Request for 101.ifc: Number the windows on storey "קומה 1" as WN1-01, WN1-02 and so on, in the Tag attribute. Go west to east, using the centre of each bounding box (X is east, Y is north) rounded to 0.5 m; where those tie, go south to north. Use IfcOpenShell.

First a look at what the model holds.

```python
import ifcopenshell
import ifcopenshell.util.element
import ifcopenshell.util.placement

model = ifcopenshell.open("101.ifc")
print(model.schema)
storey = next(s for s in model.by_type("IfcBuildingStorey") if s.Name == "קומה 1")
windows = [e for e in ifcopenshell.util.element.get_decomposition(storey) if e.is_a("IfcWindow")]
for e in sorted(windows, key=lambda e: e.id()):
    origin = ifcopenshell.util.placement.get_local_placement(e.ObjectPlacement)[:3, 3]
    print(e.id(), e.Tag, e.Name, origin.round(2) + 0.0, sep=" | ")
```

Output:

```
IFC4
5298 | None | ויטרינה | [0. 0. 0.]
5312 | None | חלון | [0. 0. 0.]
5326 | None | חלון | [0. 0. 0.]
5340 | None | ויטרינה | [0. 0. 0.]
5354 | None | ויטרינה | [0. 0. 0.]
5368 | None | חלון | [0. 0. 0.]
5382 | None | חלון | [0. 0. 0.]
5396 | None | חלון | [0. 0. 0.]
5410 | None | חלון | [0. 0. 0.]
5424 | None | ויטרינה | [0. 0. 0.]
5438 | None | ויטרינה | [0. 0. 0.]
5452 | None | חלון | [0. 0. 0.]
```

```python
import ifcopenshell
import ifcopenshell.geom
import ifcopenshell.util.element
import ifcopenshell.util.shape

model = ifcopenshell.open("101.ifc")
settings = ifcopenshell.geom.settings()
settings.set("use-world-coords", True)


def centre(element):
    shape = ifcopenshell.geom.create_shape(settings, element)
    return ifcopenshell.util.shape.get_bbox_centroid(shape.geometry)


storey = next(s for s in model.by_type("IfcBuildingStorey") if s.Name == "קומה 1")
windows = [e for e in ifcopenshell.util.element.get_decomposition(storey) if e.is_a("IfcWindow")]

# Insertion points can sit at a corner or the storey origin, so sort by the geometry (in metres).
centres = {e: centre(e) for e in windows}
windows.sort(key=lambda e: (round(centres[e][0] / 0.5), centres[e][1]))

for i, e in enumerate(windows, start=1):
    number = f"WN1-{i:02d}"
    e.Tag = number
    print(e.id(), number)

model.write("101-out.ifc")
```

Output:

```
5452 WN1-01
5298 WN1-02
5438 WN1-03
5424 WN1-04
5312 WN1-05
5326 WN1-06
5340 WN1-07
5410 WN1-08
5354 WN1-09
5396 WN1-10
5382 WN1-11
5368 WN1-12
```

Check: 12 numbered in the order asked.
